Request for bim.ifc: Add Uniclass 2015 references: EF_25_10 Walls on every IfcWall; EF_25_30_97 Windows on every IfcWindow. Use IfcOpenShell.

First a look at what the model holds.

```python
import ifcopenshell

model = ifcopenshell.open("bim.ifc")
print(model.schema)
print("classifications:", [c.Name for c in model.by_type("IfcClassification")])
for ifc_class in ("IfcDoor", "IfcRoof", "IfcStair", "IfcWall", "IfcWindow"):
    print(ifc_class, len(model.by_type(ifc_class)))
```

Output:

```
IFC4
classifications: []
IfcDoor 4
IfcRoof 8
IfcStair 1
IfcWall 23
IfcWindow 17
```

```python
import ifcopenshell
import ifcopenshell.api.classification

model = ifcopenshell.open("bim.ifc")

system = ifcopenshell.api.classification.add_classification(model, classification="Uniclass 2015")

codes = {
    "IfcWall": ("EF_25_10", "Walls"),
    "IfcWindow": ("EF_25_30_97", "Windows"),
}
for ifc_class, (code, name) in codes.items():
    products = model.by_type(ifc_class)
    ifcopenshell.api.classification.add_reference(
        model, products=products, classification=system, identification=code, name=name
    )
    print(code, len(products))

model.write("bim-out.ifc")
```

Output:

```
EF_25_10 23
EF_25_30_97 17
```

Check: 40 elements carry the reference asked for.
